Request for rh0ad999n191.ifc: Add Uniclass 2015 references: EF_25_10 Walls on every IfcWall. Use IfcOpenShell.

First a look at what the model holds.

```python
import ifcopenshell

model = ifcopenshell.open("rh0ad999n191.ifc")
print(model.schema)
print("classifications:", [c.Name for c in model.by_type("IfcClassification")])
for ifc_class in ("IfcDoor", "IfcRoof", "IfcStair", "IfcWall", "IfcWindow"):
    print(ifc_class, len(model.by_type(ifc_class)))
```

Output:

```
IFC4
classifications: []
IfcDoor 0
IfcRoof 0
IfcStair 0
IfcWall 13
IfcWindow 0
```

```python
import ifcopenshell
import ifcopenshell.api.classification

model = ifcopenshell.open("rh0ad999n191.ifc")

system = ifcopenshell.api.classification.add_classification(model, classification="Uniclass 2015")

codes = {
    "IfcWall": ("EF_25_10", "Walls"),
}
for ifc_class, (code, name) in codes.items():
    products = model.by_type(ifc_class)
    ifcopenshell.api.classification.add_reference(
        model, products=products, classification=system, identification=code, name=name
    )
    print(code, len(products))

model.write("rh0ad999n191_edited.ifc")
```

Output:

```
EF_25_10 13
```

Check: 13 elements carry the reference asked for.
